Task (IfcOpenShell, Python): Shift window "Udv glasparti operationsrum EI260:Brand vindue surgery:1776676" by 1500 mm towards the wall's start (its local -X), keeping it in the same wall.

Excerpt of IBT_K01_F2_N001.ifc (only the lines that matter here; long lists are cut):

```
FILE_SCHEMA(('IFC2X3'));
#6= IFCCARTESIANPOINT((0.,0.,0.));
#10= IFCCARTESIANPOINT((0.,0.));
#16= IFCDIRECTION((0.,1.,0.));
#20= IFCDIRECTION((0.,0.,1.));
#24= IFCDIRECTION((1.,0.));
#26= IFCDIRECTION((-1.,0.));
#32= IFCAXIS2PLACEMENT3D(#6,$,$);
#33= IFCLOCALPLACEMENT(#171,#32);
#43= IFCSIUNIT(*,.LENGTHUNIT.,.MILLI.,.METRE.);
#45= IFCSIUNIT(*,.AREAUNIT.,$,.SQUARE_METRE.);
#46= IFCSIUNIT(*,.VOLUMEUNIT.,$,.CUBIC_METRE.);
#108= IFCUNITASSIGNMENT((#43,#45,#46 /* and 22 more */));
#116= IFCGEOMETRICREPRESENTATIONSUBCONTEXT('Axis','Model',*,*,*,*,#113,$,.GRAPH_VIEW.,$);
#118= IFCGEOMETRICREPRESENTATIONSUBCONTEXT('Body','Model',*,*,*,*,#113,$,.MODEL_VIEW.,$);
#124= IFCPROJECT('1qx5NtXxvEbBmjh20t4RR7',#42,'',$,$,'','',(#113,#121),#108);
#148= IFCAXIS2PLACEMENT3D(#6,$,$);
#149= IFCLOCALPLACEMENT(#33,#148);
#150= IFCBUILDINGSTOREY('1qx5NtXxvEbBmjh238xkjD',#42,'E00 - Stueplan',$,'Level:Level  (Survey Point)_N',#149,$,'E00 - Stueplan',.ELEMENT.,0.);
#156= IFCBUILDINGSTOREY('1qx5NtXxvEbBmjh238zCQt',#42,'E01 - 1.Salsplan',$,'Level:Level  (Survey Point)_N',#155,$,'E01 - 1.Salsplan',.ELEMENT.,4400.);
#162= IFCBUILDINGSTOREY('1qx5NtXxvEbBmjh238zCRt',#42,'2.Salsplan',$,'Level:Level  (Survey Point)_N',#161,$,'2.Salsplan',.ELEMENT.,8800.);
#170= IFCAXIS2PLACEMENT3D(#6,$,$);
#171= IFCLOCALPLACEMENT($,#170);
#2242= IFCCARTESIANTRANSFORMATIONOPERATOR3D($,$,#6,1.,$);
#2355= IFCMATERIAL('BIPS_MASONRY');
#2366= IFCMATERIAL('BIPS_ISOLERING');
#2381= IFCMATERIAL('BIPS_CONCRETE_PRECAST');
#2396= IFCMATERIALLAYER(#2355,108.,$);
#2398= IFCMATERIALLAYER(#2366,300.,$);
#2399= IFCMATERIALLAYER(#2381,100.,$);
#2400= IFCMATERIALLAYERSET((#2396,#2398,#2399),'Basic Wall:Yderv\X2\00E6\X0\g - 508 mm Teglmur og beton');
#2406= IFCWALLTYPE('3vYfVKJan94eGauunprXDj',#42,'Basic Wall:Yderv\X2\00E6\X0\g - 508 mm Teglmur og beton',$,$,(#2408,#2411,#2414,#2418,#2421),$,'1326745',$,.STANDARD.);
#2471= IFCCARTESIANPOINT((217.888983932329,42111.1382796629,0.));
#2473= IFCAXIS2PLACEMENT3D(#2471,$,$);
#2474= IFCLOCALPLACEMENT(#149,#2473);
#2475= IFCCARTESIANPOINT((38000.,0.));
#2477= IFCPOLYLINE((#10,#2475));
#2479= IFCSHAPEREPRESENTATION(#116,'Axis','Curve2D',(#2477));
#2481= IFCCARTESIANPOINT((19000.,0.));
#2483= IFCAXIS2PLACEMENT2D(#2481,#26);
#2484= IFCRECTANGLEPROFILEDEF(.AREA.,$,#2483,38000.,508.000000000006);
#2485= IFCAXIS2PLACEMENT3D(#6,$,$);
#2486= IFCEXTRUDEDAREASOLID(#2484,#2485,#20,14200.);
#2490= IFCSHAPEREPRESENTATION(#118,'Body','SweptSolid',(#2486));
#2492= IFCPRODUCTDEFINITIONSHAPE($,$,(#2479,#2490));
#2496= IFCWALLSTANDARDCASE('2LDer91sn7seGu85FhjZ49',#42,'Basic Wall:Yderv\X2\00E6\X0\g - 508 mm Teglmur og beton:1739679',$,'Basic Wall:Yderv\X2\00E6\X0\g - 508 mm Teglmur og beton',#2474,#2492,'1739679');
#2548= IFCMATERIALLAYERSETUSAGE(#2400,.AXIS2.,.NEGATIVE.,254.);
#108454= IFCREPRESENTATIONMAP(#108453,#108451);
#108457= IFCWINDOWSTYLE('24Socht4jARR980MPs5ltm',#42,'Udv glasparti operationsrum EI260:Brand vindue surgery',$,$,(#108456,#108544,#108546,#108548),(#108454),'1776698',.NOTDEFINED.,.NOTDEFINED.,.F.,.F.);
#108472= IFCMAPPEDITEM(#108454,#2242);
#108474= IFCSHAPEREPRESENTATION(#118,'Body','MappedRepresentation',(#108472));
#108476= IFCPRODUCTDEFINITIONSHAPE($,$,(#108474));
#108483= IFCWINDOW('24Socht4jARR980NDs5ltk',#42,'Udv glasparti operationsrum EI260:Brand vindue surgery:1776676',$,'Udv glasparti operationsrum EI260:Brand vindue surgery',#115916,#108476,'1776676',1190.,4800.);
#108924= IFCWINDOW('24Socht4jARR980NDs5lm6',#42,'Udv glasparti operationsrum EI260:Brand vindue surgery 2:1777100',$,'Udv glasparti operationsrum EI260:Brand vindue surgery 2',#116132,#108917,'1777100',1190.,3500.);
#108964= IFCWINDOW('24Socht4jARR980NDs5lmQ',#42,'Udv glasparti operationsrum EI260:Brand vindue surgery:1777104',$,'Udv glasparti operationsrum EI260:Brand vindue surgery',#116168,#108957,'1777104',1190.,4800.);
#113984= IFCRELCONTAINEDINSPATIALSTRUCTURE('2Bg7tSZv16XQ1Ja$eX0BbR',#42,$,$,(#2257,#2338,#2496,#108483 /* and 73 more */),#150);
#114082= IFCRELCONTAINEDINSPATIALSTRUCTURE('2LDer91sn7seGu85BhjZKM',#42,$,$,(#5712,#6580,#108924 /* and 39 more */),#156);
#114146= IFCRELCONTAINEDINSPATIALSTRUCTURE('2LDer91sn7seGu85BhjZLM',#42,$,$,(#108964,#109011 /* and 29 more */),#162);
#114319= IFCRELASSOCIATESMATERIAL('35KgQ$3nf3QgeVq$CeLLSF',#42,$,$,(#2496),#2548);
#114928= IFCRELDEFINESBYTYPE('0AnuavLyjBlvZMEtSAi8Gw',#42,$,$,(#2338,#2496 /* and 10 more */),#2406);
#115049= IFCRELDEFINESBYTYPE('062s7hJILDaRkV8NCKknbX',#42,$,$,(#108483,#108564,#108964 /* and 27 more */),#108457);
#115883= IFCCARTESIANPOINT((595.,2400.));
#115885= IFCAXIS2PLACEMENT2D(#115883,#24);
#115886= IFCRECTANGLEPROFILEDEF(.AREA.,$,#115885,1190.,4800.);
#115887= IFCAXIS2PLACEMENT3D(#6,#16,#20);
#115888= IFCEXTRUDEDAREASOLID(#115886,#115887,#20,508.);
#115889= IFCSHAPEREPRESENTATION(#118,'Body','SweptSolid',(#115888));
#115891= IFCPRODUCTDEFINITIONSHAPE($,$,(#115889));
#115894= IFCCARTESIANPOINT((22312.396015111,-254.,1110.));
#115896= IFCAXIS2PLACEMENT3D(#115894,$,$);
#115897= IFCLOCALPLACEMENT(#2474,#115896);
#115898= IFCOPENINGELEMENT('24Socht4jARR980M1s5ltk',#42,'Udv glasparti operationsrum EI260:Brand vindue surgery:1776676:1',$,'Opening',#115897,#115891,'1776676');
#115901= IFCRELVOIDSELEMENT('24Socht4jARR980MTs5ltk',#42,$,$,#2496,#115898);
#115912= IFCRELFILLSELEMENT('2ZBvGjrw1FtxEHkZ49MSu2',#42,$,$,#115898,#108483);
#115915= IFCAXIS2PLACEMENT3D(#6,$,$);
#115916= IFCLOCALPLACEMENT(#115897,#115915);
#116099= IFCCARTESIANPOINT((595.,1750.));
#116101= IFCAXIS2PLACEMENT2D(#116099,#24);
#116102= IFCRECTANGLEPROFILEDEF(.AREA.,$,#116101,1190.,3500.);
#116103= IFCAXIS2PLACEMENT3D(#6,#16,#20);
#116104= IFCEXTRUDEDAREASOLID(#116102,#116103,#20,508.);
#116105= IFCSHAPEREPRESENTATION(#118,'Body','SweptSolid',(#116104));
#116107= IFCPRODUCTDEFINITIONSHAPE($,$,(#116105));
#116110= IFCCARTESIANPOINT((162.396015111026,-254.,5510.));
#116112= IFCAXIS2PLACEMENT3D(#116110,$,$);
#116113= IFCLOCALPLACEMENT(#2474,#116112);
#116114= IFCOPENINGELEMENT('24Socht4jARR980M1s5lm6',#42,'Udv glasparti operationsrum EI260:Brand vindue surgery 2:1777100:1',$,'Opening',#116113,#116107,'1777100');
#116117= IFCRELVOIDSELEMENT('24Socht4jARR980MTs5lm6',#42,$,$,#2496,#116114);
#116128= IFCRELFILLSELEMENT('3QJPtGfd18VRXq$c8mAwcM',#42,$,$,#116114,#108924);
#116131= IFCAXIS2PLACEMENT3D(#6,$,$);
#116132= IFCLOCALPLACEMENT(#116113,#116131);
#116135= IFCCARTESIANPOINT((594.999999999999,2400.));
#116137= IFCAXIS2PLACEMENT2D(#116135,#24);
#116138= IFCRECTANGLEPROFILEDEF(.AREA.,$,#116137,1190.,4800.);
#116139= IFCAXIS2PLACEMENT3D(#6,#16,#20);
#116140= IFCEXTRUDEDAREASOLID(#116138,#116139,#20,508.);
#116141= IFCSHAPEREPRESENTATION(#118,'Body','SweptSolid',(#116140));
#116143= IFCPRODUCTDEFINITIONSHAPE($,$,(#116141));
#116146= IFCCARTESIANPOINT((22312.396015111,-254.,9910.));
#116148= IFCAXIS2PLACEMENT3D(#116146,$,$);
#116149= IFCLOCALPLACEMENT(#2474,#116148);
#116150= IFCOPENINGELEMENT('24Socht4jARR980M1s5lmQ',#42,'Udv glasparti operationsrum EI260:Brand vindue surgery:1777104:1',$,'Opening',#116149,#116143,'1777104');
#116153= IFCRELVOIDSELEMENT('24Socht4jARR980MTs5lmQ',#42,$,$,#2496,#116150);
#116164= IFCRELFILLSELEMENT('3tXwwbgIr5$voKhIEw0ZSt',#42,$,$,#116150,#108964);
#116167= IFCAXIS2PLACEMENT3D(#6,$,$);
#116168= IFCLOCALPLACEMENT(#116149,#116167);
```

```python
import ifcopenshell
import ifcopenshell.api.geometry
import ifcopenshell.util.placement
import ifcopenshell.util.unit

model = ifcopenshell.open("IBT_K01_F2_N001.ifc")
unit_scale = ifcopenshell.util.unit.calculate_unit_scale(model)

window = model.by_id(108483)
opening = window.FillsVoids[0].RelatingOpeningElement
wall = opening.VoidsElements[0].RelatingBuildingElement

wall_matrix = ifcopenshell.util.placement.get_local_placement(wall.ObjectPlacement)
shift = wall_matrix[:3, 0] * -1.5 / unit_scale
before = ifcopenshell.util.placement.get_local_placement(window.ObjectPlacement)[:3, 3].copy()

# The window is placed relative to its opening, so it follows when the opening moves.
matrix = ifcopenshell.util.placement.get_local_placement(opening.ObjectPlacement)
matrix[:3, 3] += shift
ifcopenshell.api.geometry.edit_object_placement(
    model, product=opening, matrix=matrix, is_si=False, should_transform_children=True
)

after = ifcopenshell.util.placement.get_local_placement(window.ObjectPlacement)[:3, 3]
print("window moved by", (after - before).round(3) + 0.0)

model.write("IBT_K01_F2_N001_v2.ifc")
```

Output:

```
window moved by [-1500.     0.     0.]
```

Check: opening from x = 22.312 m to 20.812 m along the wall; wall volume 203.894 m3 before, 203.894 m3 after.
